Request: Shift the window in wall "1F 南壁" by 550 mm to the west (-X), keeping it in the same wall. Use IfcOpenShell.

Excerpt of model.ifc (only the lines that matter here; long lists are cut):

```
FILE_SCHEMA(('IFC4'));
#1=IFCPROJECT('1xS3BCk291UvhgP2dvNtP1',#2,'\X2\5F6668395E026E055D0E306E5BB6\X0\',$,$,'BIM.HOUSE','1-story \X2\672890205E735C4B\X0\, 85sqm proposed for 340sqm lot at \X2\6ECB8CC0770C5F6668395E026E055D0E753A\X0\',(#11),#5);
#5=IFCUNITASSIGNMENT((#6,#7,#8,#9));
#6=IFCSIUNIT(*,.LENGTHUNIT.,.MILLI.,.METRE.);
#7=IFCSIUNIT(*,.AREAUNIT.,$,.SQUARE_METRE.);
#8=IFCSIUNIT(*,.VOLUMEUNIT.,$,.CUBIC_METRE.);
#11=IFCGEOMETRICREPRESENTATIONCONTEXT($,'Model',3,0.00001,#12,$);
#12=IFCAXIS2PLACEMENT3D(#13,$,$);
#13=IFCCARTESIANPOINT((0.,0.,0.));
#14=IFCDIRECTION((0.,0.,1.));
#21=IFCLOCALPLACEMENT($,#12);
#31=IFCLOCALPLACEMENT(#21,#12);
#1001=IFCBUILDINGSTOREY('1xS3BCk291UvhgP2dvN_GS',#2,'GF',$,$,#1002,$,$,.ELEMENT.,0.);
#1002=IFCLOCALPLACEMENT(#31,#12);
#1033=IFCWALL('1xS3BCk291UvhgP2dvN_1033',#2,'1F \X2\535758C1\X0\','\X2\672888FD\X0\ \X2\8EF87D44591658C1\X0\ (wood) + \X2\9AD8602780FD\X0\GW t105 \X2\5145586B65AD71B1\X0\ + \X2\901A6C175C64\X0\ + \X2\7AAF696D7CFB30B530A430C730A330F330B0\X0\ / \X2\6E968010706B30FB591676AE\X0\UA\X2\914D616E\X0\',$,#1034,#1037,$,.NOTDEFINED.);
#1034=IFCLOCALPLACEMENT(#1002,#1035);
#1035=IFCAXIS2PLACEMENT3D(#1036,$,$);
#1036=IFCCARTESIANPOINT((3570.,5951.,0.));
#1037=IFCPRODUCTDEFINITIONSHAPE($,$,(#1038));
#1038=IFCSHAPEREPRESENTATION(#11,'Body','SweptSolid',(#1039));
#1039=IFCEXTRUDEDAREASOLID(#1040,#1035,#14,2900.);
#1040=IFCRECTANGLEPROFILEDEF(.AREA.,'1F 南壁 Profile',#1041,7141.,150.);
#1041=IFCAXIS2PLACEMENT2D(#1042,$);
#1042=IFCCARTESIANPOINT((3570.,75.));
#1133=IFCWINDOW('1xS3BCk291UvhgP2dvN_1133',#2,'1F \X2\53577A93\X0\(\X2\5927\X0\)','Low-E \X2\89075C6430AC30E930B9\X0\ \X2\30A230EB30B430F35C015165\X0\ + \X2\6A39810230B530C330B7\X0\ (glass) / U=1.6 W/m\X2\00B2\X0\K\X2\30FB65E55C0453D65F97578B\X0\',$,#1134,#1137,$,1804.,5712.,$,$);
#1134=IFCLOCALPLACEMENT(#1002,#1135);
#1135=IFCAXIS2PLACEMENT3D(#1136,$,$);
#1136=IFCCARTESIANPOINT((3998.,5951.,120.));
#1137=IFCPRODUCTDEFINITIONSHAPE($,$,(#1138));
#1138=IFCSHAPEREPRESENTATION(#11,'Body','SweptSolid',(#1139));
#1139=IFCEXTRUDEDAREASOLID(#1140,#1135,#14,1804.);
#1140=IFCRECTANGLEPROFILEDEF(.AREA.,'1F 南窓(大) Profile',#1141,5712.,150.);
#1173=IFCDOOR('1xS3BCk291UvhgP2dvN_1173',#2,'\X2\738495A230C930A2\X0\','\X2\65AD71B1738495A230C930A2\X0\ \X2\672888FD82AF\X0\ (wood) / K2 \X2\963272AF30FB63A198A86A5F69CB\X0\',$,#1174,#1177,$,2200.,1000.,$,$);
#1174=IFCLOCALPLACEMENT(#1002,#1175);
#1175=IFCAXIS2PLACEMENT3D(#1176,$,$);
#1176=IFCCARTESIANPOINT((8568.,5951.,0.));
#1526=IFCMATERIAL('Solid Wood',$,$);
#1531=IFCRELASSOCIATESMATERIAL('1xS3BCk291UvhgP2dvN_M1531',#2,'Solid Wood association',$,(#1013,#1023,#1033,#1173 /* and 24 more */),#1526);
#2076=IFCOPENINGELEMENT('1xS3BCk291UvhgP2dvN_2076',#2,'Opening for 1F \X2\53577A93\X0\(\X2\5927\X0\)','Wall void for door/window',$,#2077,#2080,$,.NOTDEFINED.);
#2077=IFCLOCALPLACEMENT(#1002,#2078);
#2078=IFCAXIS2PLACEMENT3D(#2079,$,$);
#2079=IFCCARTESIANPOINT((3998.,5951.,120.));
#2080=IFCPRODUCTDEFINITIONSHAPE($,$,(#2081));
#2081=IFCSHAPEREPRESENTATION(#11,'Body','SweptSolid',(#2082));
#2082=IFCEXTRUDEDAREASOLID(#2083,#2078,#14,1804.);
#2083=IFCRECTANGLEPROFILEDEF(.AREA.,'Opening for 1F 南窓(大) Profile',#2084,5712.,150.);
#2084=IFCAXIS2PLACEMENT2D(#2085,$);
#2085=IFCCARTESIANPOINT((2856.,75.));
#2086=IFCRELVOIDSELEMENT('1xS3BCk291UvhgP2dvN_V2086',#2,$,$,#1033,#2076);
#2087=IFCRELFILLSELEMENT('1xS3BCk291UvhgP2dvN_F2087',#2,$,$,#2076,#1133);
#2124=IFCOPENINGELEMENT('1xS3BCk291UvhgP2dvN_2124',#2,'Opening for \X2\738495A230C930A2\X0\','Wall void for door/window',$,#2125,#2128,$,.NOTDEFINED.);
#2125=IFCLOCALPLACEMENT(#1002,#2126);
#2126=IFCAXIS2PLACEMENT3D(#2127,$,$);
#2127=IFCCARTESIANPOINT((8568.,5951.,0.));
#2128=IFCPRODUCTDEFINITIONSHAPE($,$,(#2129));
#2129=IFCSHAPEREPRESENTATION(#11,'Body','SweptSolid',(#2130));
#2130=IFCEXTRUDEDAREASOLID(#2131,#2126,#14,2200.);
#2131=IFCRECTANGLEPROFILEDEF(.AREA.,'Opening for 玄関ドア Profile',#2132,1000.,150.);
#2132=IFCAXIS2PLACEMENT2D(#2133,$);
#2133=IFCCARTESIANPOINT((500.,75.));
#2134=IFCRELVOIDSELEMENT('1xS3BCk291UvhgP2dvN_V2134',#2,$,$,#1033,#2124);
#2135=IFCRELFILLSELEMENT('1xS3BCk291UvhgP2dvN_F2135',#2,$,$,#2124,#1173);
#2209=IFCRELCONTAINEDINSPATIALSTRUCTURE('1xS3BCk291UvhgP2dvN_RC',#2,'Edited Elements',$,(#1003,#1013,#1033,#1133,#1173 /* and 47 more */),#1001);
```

```python
import ifcopenshell
import ifcopenshell.api.geometry
import ifcopenshell.util.placement

model = ifcopenshell.open("model.ifc")

window = model.by_guid("1xS3BCk291UvhgP2dvN_1133")
opening = window.FillsVoids[0].RelatingOpeningElement
wall = opening.VoidsElements[0].RelatingBuildingElement

wall_matrix = ifcopenshell.util.placement.get_local_placement(wall.ObjectPlacement)
shift = wall_matrix[:3, 0] * -550.0
before = ifcopenshell.util.placement.get_local_placement(window.ObjectPlacement)[:3, 3].copy()

# The window is not placed relative to its opening, so move both.
for product in (opening, window):
    matrix = ifcopenshell.util.placement.get_local_placement(product.ObjectPlacement)
    matrix[:3, 3] += shift
    ifcopenshell.api.geometry.edit_object_placement(model, product=product, matrix=matrix, is_si=False)

after = ifcopenshell.util.placement.get_local_placement(window.ObjectPlacement)[:3, 3]
print("window moved by", (after - before).round(3) + 0.0)

model.write("model_rev.ifc")
```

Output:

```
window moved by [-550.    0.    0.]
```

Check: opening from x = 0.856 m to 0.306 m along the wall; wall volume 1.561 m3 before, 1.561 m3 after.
